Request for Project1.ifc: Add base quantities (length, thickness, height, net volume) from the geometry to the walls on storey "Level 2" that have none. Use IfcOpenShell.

First a look at what the model holds.

```python
import ifcopenshell
import ifcopenshell.util.element
import ifcopenshell.util.unit

model = ifcopenshell.open("Project1.ifc")
print(model.schema)
for unit_type in ("LENGTHUNIT", "AREAUNIT", "VOLUMEUNIT"):
    print(unit_type, ifcopenshell.util.unit.calculate_unit_scale(model, unit_type))
storey = next(s for s in model.by_type("IfcBuildingStorey") if s.Name == "Level 2")
walls = [e for e in ifcopenshell.util.element.get_decomposition(storey) if e.is_a("IfcWall")]
for e in sorted(walls, key=lambda e: e.id()):
    print(e.id(), e.is_a(), e.Name, list(ifcopenshell.util.element.get_psets(e, qtos_only=True)), sep=" | ")
```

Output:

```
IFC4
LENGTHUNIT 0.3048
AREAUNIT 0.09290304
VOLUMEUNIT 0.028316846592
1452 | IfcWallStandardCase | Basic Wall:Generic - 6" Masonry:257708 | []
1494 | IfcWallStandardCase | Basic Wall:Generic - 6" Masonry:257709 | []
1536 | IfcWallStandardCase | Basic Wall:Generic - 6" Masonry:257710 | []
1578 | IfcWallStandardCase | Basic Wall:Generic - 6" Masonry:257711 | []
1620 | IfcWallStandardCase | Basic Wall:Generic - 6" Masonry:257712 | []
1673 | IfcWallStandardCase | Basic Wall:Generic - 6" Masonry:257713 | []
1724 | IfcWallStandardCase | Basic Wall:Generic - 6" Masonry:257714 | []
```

```python
import ifcopenshell
import ifcopenshell.api.pset
import ifcopenshell.geom
import ifcopenshell.util.element
import ifcopenshell.util.shape
import ifcopenshell.util.unit

model = ifcopenshell.open("Project1.ifc")
unit_scale = ifcopenshell.util.unit.calculate_unit_scale(model)
volume_scale = ifcopenshell.util.unit.calculate_unit_scale(model, "VOLUMEUNIT")
settings = ifcopenshell.geom.settings()

storey = next(s for s in model.by_type("IfcBuildingStorey") if s.Name == "Level 2")
walls = [e for e in ifcopenshell.util.element.get_decomposition(storey) if e.is_a("IfcWall")]

for e in sorted(walls, key=lambda e: e.id()):
    if ifcopenshell.util.element.get_psets(e, qtos_only=True, should_inherit=False):
        continue
    # Geometry comes back in metres, in the element's own axes.
    shape = ifcopenshell.geom.create_shape(settings, e)
    values = {
        "Length": ifcopenshell.util.shape.get_x(shape.geometry) / unit_scale,
        "Width": ifcopenshell.util.shape.get_y(shape.geometry) / unit_scale,
        "Height": ifcopenshell.util.shape.get_z(shape.geometry) / unit_scale,
        "NetVolume": ifcopenshell.util.shape.get_volume(shape.geometry) / volume_scale,
    }
    qto = ifcopenshell.api.pset.add_qto(model, product=e, name="Qto_WallBaseQuantities")
    ifcopenshell.api.pset.edit_qto(model, qto=qto, properties=values)
    print(e.id(), {k: round(v, 3) for k, v in values.items()})

model.write("Project1_rev.ifc")
```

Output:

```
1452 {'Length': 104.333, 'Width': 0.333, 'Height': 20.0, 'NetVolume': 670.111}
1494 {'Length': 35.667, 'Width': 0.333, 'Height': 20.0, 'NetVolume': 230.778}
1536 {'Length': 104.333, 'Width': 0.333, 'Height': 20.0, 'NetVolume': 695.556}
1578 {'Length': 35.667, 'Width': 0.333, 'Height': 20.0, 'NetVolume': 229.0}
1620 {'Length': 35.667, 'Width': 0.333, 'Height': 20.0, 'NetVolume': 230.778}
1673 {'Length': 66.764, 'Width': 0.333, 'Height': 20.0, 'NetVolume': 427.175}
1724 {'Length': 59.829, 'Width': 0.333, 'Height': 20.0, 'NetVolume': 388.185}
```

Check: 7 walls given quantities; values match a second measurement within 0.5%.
